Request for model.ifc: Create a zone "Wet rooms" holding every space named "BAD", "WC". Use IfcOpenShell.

First a look at what the model holds.

```python
import ifcopenshell

model = ifcopenshell.open("model.ifc")
print(model.schema)
seen = {}
for space in model.by_type("IfcSpace"):
    seen[space.LongName] = seen.get(space.LongName, 0) + 1
for name, count in sorted(seen.items(), key=str):
    print(count, "x", name)
print("zones:", [z.Name for z in model.by_type("IfcZone")][:20])
```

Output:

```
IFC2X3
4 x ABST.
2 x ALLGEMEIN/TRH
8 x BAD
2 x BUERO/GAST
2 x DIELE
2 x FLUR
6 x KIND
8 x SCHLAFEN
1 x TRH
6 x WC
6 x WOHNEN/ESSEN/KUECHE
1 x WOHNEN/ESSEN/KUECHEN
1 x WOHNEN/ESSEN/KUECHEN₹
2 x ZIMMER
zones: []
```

```python
import ifcopenshell
import ifcopenshell.api.group
import ifcopenshell.api.root

model = ifcopenshell.open("model.ifc")

names = {"BAD", "WC"}
spaces = [s for s in model.by_type("IfcSpace") if s.LongName in names]

zone = ifcopenshell.api.root.create_entity(model, ifc_class="IfcZone", name="Wet rooms")
ifcopenshell.api.group.assign_group(model, products=spaces, group=zone)
print(len(spaces), "spaces in", zone.Name)

model.write("model_updated.ifc")
```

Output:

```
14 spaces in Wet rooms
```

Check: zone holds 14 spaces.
